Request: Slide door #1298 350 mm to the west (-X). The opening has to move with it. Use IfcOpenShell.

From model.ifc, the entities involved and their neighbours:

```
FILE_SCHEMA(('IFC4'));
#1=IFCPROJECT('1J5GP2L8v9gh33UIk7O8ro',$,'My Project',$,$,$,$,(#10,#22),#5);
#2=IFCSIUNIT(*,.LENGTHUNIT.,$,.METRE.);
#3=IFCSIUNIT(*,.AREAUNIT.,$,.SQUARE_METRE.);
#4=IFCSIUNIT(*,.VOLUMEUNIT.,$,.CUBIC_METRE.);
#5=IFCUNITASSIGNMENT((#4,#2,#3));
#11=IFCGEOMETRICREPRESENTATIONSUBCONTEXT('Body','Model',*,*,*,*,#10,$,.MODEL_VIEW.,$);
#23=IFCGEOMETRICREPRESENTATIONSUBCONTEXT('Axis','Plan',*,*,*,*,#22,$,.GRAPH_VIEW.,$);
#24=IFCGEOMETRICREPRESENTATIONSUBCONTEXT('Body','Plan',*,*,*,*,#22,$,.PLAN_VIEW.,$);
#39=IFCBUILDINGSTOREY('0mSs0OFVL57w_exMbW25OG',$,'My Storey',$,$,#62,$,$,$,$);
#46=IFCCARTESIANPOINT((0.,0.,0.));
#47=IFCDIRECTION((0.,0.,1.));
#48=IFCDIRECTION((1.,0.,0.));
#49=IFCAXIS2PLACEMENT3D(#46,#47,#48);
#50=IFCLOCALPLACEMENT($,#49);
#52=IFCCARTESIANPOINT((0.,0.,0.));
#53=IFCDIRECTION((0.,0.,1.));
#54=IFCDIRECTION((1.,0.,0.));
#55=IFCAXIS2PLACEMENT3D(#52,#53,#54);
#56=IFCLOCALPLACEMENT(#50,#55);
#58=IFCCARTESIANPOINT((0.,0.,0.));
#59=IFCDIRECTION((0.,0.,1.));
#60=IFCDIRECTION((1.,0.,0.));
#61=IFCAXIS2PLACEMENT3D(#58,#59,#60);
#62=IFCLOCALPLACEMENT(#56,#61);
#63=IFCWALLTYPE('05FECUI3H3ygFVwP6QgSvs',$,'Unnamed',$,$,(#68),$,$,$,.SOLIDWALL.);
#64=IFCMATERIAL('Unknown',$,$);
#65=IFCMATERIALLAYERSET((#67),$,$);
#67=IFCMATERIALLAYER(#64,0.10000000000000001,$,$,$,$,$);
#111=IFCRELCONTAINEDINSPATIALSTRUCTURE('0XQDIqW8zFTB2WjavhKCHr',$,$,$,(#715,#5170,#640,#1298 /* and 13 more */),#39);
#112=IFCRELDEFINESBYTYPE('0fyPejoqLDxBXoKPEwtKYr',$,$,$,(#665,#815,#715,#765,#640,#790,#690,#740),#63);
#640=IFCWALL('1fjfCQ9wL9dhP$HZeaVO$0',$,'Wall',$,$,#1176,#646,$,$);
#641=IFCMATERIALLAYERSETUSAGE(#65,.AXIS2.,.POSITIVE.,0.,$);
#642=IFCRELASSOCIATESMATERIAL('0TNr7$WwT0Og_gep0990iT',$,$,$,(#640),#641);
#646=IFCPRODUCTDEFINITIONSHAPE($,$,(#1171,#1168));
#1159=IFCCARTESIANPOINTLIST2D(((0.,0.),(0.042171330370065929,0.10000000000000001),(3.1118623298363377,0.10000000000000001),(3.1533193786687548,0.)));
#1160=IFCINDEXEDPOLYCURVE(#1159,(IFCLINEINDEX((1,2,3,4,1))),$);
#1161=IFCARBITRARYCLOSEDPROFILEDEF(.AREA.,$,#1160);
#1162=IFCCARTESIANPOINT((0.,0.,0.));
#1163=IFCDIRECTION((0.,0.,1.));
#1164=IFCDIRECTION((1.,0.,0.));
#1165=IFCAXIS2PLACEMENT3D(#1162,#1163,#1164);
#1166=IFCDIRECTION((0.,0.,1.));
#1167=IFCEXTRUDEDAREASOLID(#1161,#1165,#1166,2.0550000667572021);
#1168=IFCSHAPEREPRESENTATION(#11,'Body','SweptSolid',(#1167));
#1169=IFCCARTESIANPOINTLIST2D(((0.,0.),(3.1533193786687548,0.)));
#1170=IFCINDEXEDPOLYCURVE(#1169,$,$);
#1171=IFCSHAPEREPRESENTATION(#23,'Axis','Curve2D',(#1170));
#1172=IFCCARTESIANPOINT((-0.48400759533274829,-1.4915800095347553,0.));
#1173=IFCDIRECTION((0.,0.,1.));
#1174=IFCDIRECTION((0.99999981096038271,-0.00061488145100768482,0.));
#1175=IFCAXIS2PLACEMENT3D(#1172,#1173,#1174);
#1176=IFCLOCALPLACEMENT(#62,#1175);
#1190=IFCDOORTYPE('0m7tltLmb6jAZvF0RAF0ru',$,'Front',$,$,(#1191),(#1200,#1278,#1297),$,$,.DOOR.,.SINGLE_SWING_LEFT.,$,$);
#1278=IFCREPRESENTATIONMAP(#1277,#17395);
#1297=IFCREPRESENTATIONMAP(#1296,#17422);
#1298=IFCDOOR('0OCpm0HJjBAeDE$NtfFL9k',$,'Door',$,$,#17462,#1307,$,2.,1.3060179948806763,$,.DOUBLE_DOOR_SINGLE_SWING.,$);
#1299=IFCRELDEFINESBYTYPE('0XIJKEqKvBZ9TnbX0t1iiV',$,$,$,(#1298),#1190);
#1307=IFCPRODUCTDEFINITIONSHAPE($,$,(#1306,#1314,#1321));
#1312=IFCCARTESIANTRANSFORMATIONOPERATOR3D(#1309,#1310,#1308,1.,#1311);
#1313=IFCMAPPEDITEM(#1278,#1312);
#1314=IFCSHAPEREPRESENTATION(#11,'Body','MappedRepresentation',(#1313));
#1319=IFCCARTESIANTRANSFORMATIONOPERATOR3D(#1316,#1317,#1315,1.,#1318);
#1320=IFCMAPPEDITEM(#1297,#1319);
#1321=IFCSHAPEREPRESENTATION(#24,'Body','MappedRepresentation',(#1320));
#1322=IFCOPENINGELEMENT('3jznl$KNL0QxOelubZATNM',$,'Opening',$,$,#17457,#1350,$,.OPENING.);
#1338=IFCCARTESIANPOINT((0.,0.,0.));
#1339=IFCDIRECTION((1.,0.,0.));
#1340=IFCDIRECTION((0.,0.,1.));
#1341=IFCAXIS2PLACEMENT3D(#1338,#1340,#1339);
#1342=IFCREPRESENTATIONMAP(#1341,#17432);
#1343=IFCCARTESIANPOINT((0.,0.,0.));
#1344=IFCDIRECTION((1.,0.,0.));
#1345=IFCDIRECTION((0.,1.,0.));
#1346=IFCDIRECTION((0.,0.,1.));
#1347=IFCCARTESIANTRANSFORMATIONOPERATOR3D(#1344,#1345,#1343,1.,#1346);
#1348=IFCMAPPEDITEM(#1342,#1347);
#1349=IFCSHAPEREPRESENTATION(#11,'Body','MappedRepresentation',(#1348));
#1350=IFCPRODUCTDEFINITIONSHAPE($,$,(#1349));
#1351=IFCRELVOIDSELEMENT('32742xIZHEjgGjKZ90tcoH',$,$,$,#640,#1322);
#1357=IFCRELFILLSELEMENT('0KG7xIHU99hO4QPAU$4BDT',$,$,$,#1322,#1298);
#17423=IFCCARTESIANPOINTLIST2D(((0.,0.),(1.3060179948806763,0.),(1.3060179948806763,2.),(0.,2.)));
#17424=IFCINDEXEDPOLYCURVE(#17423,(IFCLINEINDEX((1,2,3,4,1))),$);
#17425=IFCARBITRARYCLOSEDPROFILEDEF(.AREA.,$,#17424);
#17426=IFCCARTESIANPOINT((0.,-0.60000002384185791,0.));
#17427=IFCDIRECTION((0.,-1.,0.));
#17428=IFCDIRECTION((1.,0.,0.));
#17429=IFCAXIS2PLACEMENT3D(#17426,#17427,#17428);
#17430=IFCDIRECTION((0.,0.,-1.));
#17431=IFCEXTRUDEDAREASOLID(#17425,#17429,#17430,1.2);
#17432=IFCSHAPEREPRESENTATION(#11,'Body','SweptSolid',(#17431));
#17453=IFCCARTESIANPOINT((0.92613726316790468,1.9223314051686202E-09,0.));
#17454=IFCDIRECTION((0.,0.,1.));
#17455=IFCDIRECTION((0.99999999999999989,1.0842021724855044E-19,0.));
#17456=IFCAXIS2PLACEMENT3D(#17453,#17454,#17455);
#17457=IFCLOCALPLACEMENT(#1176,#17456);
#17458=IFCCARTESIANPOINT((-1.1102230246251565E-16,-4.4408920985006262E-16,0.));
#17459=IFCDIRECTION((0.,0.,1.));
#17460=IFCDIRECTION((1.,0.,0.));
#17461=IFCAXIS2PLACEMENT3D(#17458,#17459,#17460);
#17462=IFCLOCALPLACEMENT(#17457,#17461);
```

```python
import ifcopenshell
import ifcopenshell.api.geometry
import ifcopenshell.util.placement

model = ifcopenshell.open("model.ifc")

door = model.by_guid("0OCpm0HJjBAeDE$NtfFL9k")
opening = door.FillsVoids[0].RelatingOpeningElement
wall = opening.VoidsElements[0].RelatingBuildingElement

wall_matrix = ifcopenshell.util.placement.get_local_placement(wall.ObjectPlacement)
shift = wall_matrix[:3, 0] * -0.35
before = ifcopenshell.util.placement.get_local_placement(door.ObjectPlacement)[:3, 3].copy()

# The door is placed relative to its opening, so it follows when the opening moves.
matrix = ifcopenshell.util.placement.get_local_placement(opening.ObjectPlacement)
matrix[:3, 3] += shift
ifcopenshell.api.geometry.edit_object_placement(
    model, product=opening, matrix=matrix, is_si=False, should_transform_children=True
)

after = ifcopenshell.util.placement.get_local_placement(door.ObjectPlacement)[:3, 3]
print("door moved by", (after - before).round(3) + 0.0)

model.write("model_rev.ifc")
```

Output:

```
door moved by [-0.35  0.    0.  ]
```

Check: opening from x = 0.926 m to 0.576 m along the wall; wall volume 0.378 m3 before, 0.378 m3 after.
